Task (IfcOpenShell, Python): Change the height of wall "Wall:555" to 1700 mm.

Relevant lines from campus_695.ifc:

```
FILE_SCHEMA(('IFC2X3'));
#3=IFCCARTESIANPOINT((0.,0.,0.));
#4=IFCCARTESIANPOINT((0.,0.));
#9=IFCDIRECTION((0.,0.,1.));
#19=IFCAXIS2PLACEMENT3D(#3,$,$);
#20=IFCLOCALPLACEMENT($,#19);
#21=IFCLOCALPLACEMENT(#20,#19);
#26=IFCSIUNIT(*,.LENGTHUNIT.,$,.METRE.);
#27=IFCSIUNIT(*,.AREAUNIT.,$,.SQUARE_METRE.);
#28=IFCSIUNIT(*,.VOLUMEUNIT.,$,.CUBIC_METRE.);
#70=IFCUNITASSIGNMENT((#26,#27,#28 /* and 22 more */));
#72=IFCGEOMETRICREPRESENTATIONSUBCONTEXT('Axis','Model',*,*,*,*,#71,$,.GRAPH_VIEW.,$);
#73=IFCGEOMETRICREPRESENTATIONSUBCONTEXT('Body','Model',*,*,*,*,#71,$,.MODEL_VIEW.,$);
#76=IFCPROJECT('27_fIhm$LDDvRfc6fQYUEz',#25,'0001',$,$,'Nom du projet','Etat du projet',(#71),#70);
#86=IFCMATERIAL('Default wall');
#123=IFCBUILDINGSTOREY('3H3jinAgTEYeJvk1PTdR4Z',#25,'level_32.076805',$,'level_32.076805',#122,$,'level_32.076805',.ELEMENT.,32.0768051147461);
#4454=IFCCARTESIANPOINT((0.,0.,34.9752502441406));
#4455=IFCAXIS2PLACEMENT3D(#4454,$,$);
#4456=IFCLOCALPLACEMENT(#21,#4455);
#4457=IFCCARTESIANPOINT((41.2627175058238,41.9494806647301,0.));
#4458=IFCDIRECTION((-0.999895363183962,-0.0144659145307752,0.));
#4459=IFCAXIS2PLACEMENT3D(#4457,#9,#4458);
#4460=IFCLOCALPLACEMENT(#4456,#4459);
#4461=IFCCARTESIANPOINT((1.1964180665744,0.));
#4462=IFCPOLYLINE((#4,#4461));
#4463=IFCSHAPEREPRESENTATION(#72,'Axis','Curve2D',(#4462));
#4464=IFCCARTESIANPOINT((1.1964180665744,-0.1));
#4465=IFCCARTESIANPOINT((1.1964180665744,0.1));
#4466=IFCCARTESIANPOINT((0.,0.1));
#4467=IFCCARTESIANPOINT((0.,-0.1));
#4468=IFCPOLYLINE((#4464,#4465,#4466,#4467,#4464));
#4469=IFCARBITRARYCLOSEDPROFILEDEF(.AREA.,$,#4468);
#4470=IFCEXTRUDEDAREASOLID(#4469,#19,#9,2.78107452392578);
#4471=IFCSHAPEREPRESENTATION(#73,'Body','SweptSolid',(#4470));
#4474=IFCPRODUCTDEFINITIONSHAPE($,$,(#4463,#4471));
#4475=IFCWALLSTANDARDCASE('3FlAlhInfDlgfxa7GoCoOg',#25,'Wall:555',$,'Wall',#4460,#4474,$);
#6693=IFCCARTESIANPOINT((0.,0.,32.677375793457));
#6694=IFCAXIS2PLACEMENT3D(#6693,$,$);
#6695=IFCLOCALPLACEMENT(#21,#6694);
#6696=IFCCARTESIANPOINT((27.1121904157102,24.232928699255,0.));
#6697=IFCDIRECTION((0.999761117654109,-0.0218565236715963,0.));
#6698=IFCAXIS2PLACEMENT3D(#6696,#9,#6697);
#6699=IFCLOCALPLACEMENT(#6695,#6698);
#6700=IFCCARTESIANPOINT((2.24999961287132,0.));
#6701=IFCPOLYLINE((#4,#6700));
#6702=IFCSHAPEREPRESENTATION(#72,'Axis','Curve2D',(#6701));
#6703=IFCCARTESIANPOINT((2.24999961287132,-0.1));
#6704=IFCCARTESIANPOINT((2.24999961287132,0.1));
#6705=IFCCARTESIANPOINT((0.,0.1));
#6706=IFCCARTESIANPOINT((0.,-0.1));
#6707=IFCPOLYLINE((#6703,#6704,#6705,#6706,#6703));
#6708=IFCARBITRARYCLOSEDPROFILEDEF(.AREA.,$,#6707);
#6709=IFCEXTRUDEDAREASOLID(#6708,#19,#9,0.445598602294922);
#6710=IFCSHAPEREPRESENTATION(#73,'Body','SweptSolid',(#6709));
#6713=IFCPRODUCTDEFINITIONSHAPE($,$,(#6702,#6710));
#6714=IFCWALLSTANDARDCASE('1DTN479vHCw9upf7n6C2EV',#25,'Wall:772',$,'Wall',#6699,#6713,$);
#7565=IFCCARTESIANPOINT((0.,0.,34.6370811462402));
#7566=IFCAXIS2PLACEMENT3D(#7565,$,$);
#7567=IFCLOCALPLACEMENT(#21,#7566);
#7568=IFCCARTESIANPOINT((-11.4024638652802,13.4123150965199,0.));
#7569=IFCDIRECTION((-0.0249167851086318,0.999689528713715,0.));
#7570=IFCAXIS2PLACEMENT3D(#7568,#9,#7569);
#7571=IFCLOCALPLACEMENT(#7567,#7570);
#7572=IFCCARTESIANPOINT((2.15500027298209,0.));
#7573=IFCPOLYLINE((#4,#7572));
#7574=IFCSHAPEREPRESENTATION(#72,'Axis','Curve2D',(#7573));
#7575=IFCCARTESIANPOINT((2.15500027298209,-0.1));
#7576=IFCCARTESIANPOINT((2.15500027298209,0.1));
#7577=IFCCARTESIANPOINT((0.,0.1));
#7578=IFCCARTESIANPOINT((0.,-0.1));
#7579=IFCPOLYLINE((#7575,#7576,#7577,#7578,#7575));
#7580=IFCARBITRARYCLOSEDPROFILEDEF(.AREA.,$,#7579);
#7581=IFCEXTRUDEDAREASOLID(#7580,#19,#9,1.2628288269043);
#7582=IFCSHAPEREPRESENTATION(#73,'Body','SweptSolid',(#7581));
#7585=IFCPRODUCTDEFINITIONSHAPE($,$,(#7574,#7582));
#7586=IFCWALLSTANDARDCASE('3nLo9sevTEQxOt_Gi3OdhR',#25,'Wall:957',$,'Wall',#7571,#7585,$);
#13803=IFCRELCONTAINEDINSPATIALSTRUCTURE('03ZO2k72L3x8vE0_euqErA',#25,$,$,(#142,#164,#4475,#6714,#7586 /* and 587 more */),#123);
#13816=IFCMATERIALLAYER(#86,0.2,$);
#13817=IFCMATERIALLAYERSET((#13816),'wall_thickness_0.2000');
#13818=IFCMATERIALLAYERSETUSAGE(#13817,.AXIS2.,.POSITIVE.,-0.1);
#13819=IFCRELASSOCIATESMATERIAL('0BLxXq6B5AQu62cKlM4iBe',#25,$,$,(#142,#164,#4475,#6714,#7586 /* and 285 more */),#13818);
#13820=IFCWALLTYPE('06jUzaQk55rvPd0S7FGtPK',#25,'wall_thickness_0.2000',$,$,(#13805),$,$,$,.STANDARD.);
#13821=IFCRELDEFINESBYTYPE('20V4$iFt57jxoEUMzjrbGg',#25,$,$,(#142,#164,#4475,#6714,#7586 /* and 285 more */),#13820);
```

```python
import ifcopenshell
import ifcopenshell.geom
import ifcopenshell.util.representation
import ifcopenshell.util.shape
import ifcopenshell.util.unit

model = ifcopenshell.open("campus_695.ifc")
unit_scale = ifcopenshell.util.unit.calculate_unit_scale(model)
settings = ifcopenshell.geom.settings()


def volume(element):
    """Net volume in cubic metres, openings subtracted."""
    shape = ifcopenshell.geom.create_shape(settings, element)
    return ifcopenshell.util.shape.get_volume(shape.geometry)


wall = model.by_guid("3FlAlhInfDlgfxa7GoCoOg")
before = volume(wall)

body = ifcopenshell.util.representation.get_representation(wall, "Model", "Body")
solid = body.Items[0]
old_height = solid.Depth
solid.Depth = 1.7 / unit_scale
after = volume(wall)

print(f"height {old_height:g} -> {solid.Depth:g}, volume {before:.3f} -> {after:.3f} m3")

model.write("campus_695_rev.ifc")
```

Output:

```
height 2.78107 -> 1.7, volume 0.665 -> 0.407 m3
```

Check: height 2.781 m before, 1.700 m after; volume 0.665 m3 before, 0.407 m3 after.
